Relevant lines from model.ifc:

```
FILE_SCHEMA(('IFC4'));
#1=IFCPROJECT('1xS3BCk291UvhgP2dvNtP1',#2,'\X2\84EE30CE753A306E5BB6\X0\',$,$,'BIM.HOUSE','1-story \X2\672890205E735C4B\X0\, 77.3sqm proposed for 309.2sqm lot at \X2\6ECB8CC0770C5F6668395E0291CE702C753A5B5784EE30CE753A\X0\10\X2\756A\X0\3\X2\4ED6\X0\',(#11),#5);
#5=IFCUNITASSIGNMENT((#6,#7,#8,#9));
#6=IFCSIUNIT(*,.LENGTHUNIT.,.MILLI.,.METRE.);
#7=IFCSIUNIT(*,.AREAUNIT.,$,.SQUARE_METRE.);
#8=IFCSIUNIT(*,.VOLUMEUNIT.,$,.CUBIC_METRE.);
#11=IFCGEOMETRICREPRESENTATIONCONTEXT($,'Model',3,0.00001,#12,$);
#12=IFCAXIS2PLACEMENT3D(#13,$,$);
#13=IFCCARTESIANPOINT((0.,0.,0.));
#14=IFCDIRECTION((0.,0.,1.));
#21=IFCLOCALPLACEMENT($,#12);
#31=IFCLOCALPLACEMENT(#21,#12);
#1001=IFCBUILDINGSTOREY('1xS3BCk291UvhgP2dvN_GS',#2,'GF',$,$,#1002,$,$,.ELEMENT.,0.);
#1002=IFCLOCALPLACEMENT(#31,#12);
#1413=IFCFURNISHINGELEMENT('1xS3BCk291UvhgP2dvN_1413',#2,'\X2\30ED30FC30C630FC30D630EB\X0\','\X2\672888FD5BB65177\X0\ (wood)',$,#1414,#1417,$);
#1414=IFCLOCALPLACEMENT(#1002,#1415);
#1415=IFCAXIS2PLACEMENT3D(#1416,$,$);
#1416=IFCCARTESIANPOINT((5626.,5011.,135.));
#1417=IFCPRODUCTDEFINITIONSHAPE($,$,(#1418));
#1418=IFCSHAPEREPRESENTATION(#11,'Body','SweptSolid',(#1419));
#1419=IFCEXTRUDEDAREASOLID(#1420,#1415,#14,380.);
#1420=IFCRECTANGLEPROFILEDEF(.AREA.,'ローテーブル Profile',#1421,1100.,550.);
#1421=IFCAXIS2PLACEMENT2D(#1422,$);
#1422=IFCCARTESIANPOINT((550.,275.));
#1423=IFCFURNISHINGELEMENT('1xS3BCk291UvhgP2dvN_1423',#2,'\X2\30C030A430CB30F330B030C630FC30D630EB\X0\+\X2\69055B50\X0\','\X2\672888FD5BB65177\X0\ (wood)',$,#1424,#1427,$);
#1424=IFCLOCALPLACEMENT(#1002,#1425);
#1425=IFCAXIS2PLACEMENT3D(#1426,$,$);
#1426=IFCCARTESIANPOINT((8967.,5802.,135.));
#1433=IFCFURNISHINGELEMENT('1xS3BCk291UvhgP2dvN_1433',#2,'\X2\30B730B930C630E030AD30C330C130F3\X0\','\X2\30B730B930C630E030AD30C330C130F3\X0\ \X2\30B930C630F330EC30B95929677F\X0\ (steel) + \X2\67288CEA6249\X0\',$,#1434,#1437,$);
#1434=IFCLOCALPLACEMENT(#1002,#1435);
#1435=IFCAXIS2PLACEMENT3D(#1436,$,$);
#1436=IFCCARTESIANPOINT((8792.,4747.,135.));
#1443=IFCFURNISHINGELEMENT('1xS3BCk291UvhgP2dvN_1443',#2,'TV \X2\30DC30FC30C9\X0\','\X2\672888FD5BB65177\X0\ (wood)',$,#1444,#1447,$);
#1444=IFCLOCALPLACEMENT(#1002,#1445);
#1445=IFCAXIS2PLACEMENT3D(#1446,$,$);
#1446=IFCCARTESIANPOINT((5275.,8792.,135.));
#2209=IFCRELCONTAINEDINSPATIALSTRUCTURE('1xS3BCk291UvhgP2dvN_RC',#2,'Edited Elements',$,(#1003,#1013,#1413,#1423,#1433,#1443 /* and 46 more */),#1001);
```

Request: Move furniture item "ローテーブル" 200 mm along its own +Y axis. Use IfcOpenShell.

```python
import ifcopenshell
import ifcopenshell.api.geometry
import ifcopenshell.util.placement
import ifcopenshell.util.unit

model = ifcopenshell.open("model.ifc")
unit_scale = ifcopenshell.util.unit.calculate_unit_scale(model)

item = model.by_guid("1xS3BCk291UvhgP2dvN_1413")
matrix = ifcopenshell.util.placement.get_local_placement(item.ObjectPlacement)
matrix[:3, 3] += matrix[:3, 1] * 0.2 / unit_scale
ifcopenshell.api.geometry.edit_object_placement(model, product=item, matrix=matrix, is_si=False)

print(ifcopenshell.util.placement.get_local_placement(item.ObjectPlacement).round(3) + 0.0)

model.write("model_edited.ifc")
```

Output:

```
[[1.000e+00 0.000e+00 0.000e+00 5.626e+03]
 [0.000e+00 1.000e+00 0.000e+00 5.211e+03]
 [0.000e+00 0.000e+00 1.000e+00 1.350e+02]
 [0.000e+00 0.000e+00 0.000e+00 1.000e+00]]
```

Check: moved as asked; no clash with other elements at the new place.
